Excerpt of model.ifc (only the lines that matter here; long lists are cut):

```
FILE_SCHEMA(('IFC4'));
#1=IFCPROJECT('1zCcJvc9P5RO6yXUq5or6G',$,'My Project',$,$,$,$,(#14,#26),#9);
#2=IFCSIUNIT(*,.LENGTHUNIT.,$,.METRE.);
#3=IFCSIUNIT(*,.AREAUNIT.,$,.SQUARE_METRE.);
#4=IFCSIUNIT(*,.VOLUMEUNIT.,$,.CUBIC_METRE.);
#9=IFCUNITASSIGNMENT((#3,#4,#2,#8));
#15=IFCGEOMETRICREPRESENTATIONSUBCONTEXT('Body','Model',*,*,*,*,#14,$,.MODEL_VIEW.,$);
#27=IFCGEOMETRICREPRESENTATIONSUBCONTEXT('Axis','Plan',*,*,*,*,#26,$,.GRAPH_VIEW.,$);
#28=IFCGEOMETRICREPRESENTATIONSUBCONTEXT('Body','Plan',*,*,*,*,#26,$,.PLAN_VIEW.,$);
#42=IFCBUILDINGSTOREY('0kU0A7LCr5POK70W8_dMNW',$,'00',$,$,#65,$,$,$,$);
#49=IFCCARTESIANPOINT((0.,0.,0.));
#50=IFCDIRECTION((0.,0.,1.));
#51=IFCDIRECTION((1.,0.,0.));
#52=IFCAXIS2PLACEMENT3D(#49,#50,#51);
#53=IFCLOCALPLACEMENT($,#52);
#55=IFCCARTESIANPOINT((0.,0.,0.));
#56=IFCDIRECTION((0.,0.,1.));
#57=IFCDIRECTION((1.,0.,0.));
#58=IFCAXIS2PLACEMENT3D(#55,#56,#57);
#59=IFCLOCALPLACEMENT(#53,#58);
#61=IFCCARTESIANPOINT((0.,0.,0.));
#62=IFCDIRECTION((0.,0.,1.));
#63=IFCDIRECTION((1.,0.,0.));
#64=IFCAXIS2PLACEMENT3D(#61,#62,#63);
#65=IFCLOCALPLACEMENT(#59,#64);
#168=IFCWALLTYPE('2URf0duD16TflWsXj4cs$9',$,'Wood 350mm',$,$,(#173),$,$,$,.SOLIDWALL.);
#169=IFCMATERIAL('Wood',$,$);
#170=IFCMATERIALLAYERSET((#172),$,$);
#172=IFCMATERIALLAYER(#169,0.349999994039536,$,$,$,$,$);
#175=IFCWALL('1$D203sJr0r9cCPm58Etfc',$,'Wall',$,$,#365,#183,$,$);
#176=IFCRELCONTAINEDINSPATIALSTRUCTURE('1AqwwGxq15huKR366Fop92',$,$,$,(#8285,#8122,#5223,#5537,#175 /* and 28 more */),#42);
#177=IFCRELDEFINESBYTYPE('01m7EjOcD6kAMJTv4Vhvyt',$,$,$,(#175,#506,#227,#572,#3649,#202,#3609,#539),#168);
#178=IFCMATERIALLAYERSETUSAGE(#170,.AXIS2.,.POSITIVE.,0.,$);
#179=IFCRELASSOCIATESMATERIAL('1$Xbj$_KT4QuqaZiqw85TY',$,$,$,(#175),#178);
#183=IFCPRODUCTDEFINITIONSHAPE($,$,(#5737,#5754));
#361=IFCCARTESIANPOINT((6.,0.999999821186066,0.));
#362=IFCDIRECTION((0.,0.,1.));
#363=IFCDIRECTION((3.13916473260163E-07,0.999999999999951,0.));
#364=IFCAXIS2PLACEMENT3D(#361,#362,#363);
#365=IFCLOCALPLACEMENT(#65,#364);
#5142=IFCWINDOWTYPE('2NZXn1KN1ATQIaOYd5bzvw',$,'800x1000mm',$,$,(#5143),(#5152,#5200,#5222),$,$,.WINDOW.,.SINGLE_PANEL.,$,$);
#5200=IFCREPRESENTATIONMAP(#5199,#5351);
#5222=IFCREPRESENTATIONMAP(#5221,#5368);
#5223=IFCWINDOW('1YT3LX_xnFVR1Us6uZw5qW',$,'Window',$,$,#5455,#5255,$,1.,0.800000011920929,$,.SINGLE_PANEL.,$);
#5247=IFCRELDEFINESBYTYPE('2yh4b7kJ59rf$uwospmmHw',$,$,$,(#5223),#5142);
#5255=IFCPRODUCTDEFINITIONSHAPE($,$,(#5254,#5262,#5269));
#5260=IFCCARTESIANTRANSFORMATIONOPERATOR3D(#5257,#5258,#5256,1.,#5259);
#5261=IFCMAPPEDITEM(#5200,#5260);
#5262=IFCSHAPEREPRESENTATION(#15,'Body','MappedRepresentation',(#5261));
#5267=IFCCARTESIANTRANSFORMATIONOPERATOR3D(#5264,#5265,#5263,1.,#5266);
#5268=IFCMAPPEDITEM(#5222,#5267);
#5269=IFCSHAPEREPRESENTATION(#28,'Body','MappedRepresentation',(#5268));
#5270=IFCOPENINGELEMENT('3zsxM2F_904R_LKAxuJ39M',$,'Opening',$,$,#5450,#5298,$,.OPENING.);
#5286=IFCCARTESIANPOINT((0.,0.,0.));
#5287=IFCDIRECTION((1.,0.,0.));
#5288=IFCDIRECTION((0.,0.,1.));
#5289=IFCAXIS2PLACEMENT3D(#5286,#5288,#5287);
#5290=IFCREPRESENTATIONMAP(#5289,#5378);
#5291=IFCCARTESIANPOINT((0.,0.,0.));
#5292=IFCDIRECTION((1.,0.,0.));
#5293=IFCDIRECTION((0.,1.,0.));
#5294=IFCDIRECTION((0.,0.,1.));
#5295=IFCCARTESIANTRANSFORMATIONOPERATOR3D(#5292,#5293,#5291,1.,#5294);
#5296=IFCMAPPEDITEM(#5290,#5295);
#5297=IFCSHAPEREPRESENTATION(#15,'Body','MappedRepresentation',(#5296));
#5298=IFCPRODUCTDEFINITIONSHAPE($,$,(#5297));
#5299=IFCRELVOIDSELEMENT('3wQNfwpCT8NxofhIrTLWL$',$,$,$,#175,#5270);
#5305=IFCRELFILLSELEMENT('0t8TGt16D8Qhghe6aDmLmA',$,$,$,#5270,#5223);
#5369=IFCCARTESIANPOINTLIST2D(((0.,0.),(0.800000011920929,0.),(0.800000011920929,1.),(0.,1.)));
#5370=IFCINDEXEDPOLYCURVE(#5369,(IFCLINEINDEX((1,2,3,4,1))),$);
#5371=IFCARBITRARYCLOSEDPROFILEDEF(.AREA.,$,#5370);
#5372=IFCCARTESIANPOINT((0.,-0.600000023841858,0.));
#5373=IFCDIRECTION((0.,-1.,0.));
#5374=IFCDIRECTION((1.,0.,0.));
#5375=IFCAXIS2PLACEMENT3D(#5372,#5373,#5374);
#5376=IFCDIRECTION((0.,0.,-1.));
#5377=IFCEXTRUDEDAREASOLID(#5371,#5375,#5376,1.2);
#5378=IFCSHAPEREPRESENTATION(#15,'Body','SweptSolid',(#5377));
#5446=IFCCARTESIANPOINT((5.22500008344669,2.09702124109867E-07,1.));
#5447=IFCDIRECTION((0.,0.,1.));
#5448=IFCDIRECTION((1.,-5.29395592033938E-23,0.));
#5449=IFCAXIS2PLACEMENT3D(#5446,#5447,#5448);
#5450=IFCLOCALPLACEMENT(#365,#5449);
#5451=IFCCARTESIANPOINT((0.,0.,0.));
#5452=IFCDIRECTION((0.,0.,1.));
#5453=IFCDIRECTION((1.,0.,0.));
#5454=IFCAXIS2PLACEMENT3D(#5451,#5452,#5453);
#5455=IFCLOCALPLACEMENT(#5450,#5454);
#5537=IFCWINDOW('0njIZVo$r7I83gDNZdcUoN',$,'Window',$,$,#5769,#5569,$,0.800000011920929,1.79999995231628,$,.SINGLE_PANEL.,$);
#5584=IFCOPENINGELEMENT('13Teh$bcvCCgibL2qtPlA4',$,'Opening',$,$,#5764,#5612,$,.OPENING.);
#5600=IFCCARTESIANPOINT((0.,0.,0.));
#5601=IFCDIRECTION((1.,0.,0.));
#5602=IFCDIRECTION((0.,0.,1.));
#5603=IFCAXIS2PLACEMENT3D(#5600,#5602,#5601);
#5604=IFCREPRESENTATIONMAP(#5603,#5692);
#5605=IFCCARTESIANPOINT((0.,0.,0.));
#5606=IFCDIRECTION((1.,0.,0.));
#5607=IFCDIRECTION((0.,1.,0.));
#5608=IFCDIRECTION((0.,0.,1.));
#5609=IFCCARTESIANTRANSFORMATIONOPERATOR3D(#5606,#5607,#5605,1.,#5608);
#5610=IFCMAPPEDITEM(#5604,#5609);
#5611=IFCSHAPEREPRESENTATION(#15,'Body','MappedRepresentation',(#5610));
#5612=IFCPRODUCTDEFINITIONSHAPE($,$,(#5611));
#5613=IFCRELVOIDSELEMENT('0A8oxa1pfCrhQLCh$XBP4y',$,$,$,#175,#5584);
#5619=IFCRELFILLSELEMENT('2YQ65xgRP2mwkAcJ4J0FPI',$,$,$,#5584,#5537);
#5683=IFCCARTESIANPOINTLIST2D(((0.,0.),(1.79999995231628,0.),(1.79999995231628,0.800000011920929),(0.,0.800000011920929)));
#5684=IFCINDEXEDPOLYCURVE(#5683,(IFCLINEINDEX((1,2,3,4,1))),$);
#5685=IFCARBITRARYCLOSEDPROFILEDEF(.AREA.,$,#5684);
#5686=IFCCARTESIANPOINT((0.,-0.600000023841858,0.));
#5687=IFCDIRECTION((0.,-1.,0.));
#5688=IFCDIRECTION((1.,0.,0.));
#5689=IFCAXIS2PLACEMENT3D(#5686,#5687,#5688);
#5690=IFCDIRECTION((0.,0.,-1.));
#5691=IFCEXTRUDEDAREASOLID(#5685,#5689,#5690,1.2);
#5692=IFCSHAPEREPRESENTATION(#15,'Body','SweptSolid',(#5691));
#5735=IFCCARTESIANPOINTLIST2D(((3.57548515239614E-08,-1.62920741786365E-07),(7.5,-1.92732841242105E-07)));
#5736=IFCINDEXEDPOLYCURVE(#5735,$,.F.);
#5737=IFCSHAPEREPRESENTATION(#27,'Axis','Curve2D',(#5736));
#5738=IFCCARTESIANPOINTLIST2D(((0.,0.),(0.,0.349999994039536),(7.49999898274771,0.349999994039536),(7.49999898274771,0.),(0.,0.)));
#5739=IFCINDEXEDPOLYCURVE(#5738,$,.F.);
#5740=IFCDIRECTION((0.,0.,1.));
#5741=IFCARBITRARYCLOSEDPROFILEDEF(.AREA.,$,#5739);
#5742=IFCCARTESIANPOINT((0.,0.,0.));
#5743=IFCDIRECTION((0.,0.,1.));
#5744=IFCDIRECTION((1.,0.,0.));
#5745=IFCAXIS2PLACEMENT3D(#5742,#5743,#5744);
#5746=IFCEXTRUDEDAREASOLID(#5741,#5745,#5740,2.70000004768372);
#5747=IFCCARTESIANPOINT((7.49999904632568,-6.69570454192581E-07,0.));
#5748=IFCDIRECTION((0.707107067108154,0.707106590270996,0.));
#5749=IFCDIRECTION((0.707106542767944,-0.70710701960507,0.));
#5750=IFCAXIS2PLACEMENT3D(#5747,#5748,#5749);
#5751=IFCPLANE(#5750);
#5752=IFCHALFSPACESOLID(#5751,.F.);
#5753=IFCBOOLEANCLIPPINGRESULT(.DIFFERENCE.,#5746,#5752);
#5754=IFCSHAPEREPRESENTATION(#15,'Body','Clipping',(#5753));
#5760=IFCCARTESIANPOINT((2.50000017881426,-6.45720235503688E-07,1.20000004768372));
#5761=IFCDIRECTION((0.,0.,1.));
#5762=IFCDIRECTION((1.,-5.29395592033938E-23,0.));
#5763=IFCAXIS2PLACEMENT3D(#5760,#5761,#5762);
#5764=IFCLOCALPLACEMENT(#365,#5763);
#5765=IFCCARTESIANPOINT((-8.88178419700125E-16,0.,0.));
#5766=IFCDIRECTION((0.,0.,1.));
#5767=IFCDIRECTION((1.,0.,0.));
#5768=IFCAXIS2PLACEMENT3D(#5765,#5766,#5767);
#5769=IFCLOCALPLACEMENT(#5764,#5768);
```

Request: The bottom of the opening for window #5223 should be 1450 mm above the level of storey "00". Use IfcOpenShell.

```python
import numpy as np
import ifcopenshell
import ifcopenshell.api.geometry
import ifcopenshell.geom
import ifcopenshell.util.element
import ifcopenshell.util.placement
import ifcopenshell.util.shape
import ifcopenshell.util.unit

model = ifcopenshell.open("model.ifc")
unit_scale = ifcopenshell.util.unit.calculate_unit_scale(model)

window = model.by_guid("1YT3LX_xnFVR1Us6uZw5qW")
opening = window.FillsVoids[0].RelatingOpeningElement
storey = ifcopenshell.util.element.get_container(window, ifc_class="IfcBuildingStorey")
level = ifcopenshell.util.placement.get_local_placement(storey.ObjectPlacement)[2, 3]

# The opening's origin need not be at the sill, so measure its lowest point.
shape = ifcopenshell.geom.create_shape(ifcopenshell.geom.settings(), opening)
bottom = ifcopenshell.util.shape.get_shape_bottom_elevation(shape, shape.geometry) / unit_scale
dz = level + 1.45 / unit_scale - bottom

shift = np.array([0.0, 0.0, dz])
# The window is placed relative to its opening, so it follows when the opening moves.
matrix = ifcopenshell.util.placement.get_local_placement(opening.ObjectPlacement)
matrix[:3, 3] += shift
ifcopenshell.api.geometry.edit_object_placement(
    model, product=opening, matrix=matrix, is_si=False, should_transform_children=True
)

print(f"moved by {dz * unit_scale:+.3f} m")

model.write("model_edited.ifc")
```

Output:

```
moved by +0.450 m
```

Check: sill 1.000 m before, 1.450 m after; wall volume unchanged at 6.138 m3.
